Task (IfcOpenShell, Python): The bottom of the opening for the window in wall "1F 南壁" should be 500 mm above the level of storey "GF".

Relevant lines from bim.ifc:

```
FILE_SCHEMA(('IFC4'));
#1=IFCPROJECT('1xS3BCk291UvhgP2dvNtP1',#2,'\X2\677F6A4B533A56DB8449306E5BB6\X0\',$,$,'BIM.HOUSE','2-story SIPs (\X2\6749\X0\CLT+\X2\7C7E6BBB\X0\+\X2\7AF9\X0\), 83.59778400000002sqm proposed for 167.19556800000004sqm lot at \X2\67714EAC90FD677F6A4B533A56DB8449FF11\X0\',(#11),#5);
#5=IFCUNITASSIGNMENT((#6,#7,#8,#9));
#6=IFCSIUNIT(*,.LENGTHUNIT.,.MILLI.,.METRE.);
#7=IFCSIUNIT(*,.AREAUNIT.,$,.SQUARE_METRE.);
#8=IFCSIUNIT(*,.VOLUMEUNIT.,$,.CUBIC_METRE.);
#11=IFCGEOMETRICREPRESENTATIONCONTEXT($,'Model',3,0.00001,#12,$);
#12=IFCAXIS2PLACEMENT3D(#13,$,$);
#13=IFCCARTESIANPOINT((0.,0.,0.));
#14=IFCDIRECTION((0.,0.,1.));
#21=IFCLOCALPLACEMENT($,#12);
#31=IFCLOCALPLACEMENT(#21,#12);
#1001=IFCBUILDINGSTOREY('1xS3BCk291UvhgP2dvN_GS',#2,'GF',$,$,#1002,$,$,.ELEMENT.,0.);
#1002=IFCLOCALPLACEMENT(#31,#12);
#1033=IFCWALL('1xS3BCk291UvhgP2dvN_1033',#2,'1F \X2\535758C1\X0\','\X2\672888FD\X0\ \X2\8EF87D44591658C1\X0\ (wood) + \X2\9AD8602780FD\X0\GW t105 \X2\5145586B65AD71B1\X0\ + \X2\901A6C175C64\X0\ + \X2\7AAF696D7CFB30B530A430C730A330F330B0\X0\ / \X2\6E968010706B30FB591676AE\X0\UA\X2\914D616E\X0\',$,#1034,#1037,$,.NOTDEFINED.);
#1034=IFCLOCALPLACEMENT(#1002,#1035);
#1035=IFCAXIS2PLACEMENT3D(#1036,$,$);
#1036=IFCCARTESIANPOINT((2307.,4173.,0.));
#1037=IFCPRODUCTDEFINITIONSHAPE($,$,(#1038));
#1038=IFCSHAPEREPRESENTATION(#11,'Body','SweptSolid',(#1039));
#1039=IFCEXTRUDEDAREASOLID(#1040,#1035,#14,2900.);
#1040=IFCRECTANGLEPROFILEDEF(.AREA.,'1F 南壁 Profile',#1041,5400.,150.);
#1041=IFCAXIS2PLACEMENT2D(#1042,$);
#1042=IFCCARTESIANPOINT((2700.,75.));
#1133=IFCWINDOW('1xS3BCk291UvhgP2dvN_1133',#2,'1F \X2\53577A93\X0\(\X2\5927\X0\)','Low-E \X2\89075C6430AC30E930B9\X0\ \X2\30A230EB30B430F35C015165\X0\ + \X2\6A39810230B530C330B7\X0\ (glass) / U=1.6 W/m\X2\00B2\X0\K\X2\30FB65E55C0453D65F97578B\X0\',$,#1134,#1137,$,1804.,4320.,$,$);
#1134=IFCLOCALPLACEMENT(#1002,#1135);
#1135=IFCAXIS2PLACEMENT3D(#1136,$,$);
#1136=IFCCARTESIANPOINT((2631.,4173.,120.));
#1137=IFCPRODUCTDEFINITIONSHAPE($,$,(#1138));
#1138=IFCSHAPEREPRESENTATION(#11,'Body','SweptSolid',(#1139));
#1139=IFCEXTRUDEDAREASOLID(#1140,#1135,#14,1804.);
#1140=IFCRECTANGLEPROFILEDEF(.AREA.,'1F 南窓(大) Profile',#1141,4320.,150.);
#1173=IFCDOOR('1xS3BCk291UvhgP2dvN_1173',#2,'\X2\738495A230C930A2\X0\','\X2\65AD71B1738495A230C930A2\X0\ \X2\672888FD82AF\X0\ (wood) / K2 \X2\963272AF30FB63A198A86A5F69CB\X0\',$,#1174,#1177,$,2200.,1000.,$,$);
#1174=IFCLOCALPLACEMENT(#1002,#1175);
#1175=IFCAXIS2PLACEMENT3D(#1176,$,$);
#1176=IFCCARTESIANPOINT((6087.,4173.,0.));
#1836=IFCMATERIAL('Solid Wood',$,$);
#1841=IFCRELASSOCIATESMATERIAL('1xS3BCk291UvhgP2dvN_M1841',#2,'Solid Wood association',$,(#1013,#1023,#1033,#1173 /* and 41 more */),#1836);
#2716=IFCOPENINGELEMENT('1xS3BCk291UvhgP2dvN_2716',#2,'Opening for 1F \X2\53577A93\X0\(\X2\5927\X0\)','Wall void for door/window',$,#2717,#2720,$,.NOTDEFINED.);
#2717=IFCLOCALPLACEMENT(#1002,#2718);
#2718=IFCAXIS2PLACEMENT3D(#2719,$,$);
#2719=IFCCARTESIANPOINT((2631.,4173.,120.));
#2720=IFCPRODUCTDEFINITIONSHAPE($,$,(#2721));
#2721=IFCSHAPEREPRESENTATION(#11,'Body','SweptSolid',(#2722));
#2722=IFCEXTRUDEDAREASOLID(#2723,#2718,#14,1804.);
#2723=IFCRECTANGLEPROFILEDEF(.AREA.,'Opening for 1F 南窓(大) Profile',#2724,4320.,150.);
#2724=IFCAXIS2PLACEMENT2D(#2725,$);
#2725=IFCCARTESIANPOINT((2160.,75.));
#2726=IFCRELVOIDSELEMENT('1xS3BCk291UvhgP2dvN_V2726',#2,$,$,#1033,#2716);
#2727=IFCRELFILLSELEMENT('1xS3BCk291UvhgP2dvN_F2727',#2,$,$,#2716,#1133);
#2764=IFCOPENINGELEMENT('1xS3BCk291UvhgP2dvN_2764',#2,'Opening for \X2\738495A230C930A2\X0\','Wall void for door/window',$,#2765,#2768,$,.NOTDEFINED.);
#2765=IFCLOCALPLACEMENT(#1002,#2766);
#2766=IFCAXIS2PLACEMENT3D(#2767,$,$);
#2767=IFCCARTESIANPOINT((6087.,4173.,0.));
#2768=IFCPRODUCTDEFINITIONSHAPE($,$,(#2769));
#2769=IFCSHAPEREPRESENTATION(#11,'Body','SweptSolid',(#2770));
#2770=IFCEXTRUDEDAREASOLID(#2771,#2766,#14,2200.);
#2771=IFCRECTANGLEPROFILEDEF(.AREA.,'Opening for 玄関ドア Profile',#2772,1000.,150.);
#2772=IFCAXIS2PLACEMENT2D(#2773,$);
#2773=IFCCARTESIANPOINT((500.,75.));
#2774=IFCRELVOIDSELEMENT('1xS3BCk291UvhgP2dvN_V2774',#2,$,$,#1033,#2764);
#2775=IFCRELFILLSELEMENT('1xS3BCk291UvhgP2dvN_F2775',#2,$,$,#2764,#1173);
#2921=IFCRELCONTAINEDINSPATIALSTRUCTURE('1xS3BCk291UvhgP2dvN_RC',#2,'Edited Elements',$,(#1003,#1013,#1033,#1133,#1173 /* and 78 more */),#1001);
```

```python
import numpy as np
import ifcopenshell
import ifcopenshell.api.geometry
import ifcopenshell.geom
import ifcopenshell.util.element
import ifcopenshell.util.placement
import ifcopenshell.util.shape
import ifcopenshell.util.unit

model = ifcopenshell.open("bim.ifc")
unit_scale = ifcopenshell.util.unit.calculate_unit_scale(model)

window = model.by_guid("1xS3BCk291UvhgP2dvN_1133")
opening = window.FillsVoids[0].RelatingOpeningElement
storey = ifcopenshell.util.element.get_container(window, ifc_class="IfcBuildingStorey")
level = ifcopenshell.util.placement.get_local_placement(storey.ObjectPlacement)[2, 3]

# The opening's origin need not be at the sill, so measure its lowest point.
shape = ifcopenshell.geom.create_shape(ifcopenshell.geom.settings(), opening)
bottom = ifcopenshell.util.shape.get_shape_bottom_elevation(shape, shape.geometry) / unit_scale
dz = level + 0.5 / unit_scale - bottom

shift = np.array([0.0, 0.0, dz])
# The window is not placed relative to its opening, so move both.
for product in (opening, window):
    matrix = ifcopenshell.util.placement.get_local_placement(product.ObjectPlacement)
    matrix[:3, 3] += shift
    ifcopenshell.api.geometry.edit_object_placement(model, product=product, matrix=matrix, is_si=False)

print(f"moved by {dz * unit_scale:+.3f} m")

model.write("bim_updated.ifc")
```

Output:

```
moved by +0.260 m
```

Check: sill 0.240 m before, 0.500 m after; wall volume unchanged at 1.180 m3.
